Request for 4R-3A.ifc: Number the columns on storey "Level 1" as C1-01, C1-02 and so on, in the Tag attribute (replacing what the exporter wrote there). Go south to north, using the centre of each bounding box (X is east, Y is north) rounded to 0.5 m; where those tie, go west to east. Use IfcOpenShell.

First a look at what the model holds.

```python
import ifcopenshell
import ifcopenshell.util.element
import ifcopenshell.util.placement

model = ifcopenshell.open("4R-3A.ifc")
print(model.schema)
storey = next(s for s in model.by_type("IfcBuildingStorey") if s.Name == "Level 1")
columns = [e for e in ifcopenshell.util.element.get_decomposition(storey) if e.is_a("IfcColumn")]
for e in sorted(columns, key=lambda e: e.id()):
    origin = ifcopenshell.util.placement.get_local_placement(e.ObjectPlacement)[:3, 3]
    print(e.id(), e.Tag, e.Name, origin.round(2) + 0.0, sep=" | ")
```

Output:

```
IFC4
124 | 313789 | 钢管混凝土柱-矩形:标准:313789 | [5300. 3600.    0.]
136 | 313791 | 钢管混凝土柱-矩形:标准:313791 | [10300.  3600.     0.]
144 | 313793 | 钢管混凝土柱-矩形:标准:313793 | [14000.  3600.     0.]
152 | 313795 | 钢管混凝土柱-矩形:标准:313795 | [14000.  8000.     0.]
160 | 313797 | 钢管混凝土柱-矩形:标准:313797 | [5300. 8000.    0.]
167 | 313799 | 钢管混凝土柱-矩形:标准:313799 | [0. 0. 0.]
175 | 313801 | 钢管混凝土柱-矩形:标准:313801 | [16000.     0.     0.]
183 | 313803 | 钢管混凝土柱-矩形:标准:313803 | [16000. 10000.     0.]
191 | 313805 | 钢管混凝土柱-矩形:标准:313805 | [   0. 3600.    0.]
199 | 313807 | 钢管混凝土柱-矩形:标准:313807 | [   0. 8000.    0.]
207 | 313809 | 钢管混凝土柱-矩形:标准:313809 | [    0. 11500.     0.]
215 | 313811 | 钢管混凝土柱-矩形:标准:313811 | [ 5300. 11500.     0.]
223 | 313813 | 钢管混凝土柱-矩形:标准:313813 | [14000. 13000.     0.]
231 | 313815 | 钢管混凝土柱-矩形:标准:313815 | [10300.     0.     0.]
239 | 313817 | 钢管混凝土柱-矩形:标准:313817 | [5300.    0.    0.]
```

```python
import ifcopenshell
import ifcopenshell.geom
import ifcopenshell.util.element
import ifcopenshell.util.shape

model = ifcopenshell.open("4R-3A.ifc")
settings = ifcopenshell.geom.settings()
settings.set("use-world-coords", True)


def centre(element):
    shape = ifcopenshell.geom.create_shape(settings, element)
    return ifcopenshell.util.shape.get_bbox_centroid(shape.geometry)


storey = next(s for s in model.by_type("IfcBuildingStorey") if s.Name == "Level 1")
columns = [e for e in ifcopenshell.util.element.get_decomposition(storey) if e.is_a("IfcColumn")]

# Insertion points can sit at a corner or the storey origin, so sort by the geometry (in metres).
centres = {e: centre(e) for e in columns}
columns.sort(key=lambda e: (round(centres[e][1] / 0.5), centres[e][0]))

for i, e in enumerate(columns, start=1):
    number = f"C1-{i:02d}"
    e.Tag = number
    print(e.id(), number)

model.write("4R-3A-out.ifc")
```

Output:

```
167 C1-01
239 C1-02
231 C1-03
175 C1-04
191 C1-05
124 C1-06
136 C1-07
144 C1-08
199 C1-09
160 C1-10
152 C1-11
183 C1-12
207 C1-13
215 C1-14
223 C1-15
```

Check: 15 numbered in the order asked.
